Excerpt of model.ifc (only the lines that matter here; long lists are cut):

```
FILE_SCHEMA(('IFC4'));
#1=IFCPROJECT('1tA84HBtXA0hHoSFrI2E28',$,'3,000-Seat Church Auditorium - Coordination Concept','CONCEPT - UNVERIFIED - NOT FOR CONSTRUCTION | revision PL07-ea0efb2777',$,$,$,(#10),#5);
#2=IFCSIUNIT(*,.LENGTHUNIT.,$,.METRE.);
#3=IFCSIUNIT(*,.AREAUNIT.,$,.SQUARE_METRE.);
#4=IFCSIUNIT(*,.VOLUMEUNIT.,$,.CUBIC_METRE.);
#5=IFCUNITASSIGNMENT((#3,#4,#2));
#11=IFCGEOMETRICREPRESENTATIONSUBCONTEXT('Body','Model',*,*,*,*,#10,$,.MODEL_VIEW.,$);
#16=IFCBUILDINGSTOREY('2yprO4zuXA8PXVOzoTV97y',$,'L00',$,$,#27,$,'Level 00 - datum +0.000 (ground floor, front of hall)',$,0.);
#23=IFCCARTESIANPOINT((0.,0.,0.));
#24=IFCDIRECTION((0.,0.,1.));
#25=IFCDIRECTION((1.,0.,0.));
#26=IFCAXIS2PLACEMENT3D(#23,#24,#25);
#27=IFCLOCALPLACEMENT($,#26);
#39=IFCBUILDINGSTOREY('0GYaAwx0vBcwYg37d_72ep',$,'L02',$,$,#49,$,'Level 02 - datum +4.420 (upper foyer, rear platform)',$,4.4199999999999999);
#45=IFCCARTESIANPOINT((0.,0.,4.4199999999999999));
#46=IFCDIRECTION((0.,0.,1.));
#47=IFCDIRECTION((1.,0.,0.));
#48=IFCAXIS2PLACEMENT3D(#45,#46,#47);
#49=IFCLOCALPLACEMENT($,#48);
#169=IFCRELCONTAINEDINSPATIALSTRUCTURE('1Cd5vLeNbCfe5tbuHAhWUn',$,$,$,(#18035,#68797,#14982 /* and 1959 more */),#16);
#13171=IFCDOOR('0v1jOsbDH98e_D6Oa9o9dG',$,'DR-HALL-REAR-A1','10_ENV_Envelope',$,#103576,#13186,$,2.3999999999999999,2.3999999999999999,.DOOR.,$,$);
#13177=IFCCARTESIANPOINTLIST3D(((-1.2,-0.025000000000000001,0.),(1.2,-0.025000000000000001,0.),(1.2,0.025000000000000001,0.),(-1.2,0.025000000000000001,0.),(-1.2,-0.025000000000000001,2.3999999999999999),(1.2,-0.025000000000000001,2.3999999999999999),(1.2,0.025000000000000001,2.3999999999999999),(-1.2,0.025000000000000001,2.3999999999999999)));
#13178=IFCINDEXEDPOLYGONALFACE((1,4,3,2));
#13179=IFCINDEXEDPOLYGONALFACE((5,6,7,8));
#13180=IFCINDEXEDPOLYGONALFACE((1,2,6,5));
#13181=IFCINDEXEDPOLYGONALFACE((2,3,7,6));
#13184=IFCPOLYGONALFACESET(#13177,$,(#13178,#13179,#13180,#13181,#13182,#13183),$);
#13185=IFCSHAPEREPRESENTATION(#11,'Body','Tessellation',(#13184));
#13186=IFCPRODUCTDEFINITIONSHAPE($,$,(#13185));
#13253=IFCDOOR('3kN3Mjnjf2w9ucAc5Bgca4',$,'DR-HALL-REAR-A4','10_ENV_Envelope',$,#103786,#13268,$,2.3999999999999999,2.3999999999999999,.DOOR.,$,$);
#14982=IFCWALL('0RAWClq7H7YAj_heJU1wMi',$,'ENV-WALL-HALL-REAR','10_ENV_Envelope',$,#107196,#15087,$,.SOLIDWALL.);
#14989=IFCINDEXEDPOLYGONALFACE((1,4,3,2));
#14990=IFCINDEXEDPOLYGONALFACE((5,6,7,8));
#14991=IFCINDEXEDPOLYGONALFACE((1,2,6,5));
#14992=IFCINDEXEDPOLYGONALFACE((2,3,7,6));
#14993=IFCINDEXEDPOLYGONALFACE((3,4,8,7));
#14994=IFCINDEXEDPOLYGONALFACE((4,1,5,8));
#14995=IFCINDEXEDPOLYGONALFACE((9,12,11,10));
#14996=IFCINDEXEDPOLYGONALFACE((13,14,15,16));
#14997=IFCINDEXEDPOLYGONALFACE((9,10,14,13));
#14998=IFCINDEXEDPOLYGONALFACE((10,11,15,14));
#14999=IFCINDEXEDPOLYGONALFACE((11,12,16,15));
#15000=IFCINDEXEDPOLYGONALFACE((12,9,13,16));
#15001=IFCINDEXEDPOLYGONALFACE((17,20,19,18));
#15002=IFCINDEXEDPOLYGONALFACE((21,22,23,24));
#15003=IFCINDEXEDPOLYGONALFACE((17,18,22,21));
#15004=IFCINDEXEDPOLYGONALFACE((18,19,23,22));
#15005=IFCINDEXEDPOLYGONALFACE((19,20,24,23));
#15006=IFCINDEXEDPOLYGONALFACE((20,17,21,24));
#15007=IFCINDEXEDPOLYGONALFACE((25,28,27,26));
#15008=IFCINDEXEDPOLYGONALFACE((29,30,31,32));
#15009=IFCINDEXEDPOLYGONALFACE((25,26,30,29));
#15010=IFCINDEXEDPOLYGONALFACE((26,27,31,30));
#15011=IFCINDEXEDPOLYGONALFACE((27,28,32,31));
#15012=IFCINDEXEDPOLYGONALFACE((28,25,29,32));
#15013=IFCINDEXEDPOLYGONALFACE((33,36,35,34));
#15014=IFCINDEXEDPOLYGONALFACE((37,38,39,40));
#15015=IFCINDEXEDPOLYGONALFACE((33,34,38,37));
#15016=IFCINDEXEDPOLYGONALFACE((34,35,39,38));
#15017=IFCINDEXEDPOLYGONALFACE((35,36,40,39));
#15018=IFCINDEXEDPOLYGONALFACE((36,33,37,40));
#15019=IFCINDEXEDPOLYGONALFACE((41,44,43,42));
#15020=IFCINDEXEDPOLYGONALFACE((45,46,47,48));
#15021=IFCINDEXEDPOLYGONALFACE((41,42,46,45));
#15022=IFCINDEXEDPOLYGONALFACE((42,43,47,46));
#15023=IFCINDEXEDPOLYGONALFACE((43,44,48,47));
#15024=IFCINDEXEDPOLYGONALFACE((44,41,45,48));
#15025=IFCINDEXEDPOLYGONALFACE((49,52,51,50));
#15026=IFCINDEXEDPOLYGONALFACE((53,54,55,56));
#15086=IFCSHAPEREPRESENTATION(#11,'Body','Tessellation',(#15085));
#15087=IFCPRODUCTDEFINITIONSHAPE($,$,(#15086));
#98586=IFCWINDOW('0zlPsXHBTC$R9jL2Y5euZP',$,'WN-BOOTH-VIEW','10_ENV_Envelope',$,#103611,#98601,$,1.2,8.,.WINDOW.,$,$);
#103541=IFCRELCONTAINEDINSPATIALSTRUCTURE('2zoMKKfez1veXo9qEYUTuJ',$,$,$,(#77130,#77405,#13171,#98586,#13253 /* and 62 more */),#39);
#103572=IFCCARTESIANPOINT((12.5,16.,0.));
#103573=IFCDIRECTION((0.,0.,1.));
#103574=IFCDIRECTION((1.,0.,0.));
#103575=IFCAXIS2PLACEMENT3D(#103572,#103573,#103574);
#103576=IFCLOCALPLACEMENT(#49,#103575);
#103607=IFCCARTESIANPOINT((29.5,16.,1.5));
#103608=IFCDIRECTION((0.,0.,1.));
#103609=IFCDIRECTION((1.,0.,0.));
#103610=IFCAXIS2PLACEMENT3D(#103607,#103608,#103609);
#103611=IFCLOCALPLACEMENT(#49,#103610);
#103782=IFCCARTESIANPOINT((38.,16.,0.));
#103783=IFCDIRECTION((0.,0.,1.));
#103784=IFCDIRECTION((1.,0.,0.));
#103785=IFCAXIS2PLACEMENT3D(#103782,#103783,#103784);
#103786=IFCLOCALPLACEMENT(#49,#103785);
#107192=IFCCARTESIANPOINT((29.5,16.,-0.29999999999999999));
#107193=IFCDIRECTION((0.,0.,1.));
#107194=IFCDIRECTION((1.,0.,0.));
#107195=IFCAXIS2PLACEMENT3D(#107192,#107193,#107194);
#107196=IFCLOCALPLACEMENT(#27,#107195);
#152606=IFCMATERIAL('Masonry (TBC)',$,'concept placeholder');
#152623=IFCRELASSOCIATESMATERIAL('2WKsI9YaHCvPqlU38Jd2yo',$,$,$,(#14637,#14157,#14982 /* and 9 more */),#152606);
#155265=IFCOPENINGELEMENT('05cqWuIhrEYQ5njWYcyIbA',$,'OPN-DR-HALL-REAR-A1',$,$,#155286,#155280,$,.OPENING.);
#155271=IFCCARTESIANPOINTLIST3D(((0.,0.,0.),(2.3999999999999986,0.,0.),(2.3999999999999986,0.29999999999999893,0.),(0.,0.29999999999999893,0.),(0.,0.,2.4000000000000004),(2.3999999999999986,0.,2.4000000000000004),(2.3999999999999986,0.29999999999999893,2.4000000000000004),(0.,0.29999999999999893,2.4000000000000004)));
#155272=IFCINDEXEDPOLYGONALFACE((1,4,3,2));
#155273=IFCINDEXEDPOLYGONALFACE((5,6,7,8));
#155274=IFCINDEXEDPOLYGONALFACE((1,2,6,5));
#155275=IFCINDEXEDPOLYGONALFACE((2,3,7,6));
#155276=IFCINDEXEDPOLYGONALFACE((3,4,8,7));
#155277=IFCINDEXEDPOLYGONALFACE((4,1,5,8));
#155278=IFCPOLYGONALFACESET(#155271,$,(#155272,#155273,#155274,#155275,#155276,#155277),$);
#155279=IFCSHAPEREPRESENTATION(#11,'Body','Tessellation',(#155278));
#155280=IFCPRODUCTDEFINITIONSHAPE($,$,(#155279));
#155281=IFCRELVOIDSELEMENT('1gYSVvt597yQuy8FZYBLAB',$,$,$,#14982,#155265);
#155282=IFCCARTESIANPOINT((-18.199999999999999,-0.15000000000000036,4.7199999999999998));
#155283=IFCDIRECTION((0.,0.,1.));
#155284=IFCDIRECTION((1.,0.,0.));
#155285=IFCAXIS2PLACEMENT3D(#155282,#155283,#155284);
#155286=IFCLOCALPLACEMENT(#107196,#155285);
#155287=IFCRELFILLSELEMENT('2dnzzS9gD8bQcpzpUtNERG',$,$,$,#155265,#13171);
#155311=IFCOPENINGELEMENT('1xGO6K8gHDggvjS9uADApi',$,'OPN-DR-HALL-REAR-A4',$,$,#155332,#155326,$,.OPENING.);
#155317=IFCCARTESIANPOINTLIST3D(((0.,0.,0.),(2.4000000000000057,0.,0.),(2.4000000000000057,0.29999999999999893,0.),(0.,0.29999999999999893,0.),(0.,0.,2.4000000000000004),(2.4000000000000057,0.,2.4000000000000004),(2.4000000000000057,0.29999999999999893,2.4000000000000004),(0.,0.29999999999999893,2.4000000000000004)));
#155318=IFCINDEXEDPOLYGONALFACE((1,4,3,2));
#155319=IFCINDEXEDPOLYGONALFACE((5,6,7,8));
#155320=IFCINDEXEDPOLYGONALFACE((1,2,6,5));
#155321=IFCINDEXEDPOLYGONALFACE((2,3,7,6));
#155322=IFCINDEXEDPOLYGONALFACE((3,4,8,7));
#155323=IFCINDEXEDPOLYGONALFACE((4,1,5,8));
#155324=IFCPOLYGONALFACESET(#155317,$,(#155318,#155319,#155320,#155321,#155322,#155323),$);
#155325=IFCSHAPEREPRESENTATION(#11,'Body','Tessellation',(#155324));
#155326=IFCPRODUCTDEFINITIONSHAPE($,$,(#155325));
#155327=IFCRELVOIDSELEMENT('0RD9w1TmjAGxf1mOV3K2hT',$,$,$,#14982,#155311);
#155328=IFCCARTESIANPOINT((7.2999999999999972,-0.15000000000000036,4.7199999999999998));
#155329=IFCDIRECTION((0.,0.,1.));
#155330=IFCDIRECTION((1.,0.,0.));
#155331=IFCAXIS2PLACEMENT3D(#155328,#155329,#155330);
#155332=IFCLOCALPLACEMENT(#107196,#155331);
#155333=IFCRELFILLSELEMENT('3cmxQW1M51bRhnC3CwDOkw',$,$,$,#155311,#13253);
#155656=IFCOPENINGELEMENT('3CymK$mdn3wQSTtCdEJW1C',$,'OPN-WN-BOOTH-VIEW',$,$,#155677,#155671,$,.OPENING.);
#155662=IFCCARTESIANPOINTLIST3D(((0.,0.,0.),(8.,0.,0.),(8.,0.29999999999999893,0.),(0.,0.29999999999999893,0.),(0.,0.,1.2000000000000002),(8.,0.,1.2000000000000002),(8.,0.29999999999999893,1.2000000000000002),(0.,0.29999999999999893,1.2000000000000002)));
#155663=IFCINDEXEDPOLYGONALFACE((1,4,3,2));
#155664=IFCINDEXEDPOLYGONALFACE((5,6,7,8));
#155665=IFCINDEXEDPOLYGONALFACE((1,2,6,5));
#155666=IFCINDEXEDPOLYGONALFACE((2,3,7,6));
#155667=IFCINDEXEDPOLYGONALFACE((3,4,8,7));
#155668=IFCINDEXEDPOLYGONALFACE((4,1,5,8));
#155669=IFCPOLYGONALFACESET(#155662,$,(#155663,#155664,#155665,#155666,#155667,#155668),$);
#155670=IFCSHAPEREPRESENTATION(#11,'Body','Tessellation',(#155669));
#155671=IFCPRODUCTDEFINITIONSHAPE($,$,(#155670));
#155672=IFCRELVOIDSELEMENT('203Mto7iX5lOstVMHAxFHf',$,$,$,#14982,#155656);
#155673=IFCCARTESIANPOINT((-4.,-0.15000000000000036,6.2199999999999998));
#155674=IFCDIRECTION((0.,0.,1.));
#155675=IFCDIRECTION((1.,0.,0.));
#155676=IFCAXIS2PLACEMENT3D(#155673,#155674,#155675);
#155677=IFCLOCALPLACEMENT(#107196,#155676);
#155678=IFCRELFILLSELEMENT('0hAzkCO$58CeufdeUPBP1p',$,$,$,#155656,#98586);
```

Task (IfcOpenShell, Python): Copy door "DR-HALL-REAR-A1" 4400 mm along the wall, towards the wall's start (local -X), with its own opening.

```python
import ifcopenshell
import ifcopenshell.api.feature
import ifcopenshell.api.geometry
import ifcopenshell.api.root
import ifcopenshell.geom
import ifcopenshell.util.element
import ifcopenshell.util.placement
import ifcopenshell.util.shape
import ifcopenshell.util.unit

model = ifcopenshell.open("model.ifc")
unit_scale = ifcopenshell.util.unit.calculate_unit_scale(model)
settings = ifcopenshell.geom.settings()


def volume(element):
    """Net volume in cubic metres, openings subtracted."""
    shape = ifcopenshell.geom.create_shape(settings, element)
    return ifcopenshell.util.shape.get_volume(shape.geometry)


door = model.by_guid("0v1jOsbDH98e_D6Oa9o9dG")
opening = door.FillsVoids[0].RelatingOpeningElement
wall = opening.VoidsElements[0].RelatingBuildingElement
before = volume(wall)
shift = ifcopenshell.util.placement.get_local_placement(wall.ObjectPlacement)[:3, 0] * -4.4 / unit_scale

# copy_class copies the void relationship, type, container and properties, but no geometry.
new_opening = ifcopenshell.api.root.copy_class(model, product=opening)
new_opening.Representation = ifcopenshell.util.element.copy_deep(
    model, opening.Representation, exclude=["IfcGeometricRepresentationContext", "IfcRepresentationMap"]
)
new_door = ifcopenshell.api.root.copy_class(model, product=door)
new_door.Representation = ifcopenshell.util.element.copy_deep(
    model, door.Representation, exclude=["IfcGeometricRepresentationContext", "IfcRepresentationMap"]
)
ifcopenshell.api.feature.add_filling(model, opening=new_opening, element=new_door)

for old, new in ((opening, new_opening), (door, new_door)):
    matrix = ifcopenshell.util.placement.get_local_placement(old.ObjectPlacement)
    matrix[:3, 3] += shift
    ifcopenshell.api.geometry.edit_object_placement(model, product=new, matrix=matrix, is_si=False)

after = volume(wall)

print(f"wall volume {before:.3f} -> {after:.3f} m3")

model.write("model_edited.ifc")
```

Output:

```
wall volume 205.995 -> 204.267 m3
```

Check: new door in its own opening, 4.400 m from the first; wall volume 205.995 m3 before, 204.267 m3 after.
